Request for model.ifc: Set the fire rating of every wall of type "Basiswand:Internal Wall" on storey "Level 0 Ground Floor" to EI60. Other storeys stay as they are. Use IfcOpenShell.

First a look at what the model holds.

```python
import ifcopenshell
import ifcopenshell.util.element

model = ifcopenshell.open("model.ifc")
print(model.schema)
storey = next(s for s in model.by_type("IfcBuildingStorey") if s.Name == "Level 0 Ground Floor")
walls = [e for e in ifcopenshell.util.element.get_decomposition(storey) if e.is_a("IfcWall")]
seen = {}
for e in walls:
    element_type = ifcopenshell.util.element.get_type(e)
    key = (element_type.Name if element_type != e and element_type else None, ifcopenshell.util.element.get_pset(e, "Pset_WallCommon", "FireRating"))
    seen[key] = seen.get(key, 0) + 1
for (name, value), count in sorted(seen.items(), key=str):
    print(count, "x", name, "|", value)
```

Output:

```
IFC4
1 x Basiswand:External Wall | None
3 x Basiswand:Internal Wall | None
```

```python
import ifcopenshell
import ifcopenshell.api.pset
import ifcopenshell.util.element

model = ifcopenshell.open("model.ifc")

storey = next(s for s in model.by_type("IfcBuildingStorey") if s.Name == "Level 0 Ground Floor")
walls = [e for e in ifcopenshell.util.element.get_decomposition(storey) if e.is_a("IfcWall")]

count = 0
for e in walls:
    element_type = ifcopenshell.util.element.get_type(e)
    if element_type in (None, e) or element_type.Name != "Basiswand:Internal Wall":
        continue
    # add_pset returns the element's existing set when there is one.
    pset = ifcopenshell.api.pset.add_pset(model, product=e, name="Pset_WallCommon")
    ifcopenshell.api.pset.edit_pset(model, pset=pset, properties={"FireRating": "EI60"})
    count += 1

print(count, "walls updated")

model.write("model_rev.ifc")
```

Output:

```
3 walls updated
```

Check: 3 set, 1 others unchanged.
